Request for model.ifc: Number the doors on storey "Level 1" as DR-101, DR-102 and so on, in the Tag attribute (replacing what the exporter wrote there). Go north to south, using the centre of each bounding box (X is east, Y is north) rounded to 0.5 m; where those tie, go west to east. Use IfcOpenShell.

First a look at what the model holds.

```python
import ifcopenshell
import ifcopenshell.util.element
import ifcopenshell.util.placement

model = ifcopenshell.open("model.ifc")
print(model.schema)
storey = next(s for s in model.by_type("IfcBuildingStorey") if s.Name == "Level 1")
doors = [e for e in ifcopenshell.util.element.get_decomposition(storey) if e.is_a("IfcDoor")]
for e in sorted(doors, key=lambda e: e.id()):
    origin = ifcopenshell.util.placement.get_local_placement(e.ObjectPlacement)[:3, 3]
    print(e.id(), e.Tag, e.Name, origin.round(2) + 0.0, sep=" | ")
```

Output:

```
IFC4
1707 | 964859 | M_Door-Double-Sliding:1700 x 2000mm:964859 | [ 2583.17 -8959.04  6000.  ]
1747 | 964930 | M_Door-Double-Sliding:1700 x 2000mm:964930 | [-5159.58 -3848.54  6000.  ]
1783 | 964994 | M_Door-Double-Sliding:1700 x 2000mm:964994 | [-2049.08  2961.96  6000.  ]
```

```python
import ifcopenshell
import ifcopenshell.geom
import ifcopenshell.util.element
import ifcopenshell.util.shape

model = ifcopenshell.open("model.ifc")
settings = ifcopenshell.geom.settings()
settings.set("use-world-coords", True)


def centre(element):
    shape = ifcopenshell.geom.create_shape(settings, element)
    return ifcopenshell.util.shape.get_bbox_centroid(shape.geometry)


storey = next(s for s in model.by_type("IfcBuildingStorey") if s.Name == "Level 1")
doors = [e for e in ifcopenshell.util.element.get_decomposition(storey) if e.is_a("IfcDoor")]

# Insertion points can sit at a corner or the storey origin, so sort by the geometry (in metres).
centres = {e: centre(e) for e in doors}
doors.sort(key=lambda e: (-round(centres[e][1] / 0.5), centres[e][0]))

for i, e in enumerate(doors, start=1):
    number = f"DR-1{i:02d}"
    e.Tag = number
    print(e.id(), number)

model.write("model_v2.ifc")
```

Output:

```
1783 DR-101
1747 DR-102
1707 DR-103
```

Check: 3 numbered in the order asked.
